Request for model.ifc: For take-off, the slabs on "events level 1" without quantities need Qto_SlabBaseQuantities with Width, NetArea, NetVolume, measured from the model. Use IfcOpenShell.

First a look at what the model holds.

```python
import ifcopenshell
import ifcopenshell.util.element
import ifcopenshell.util.unit

model = ifcopenshell.open("model.ifc")
print(model.schema)
for unit_type in ("LENGTHUNIT", "AREAUNIT", "VOLUMEUNIT"):
    print(unit_type, ifcopenshell.util.unit.calculate_unit_scale(model, unit_type))
storey = next(s for s in model.by_type("IfcBuildingStorey") if s.Name == "events level 1")
slabs = [e for e in ifcopenshell.util.element.get_decomposition(storey) if e.is_a("IfcSlab")]
for e in sorted(slabs, key=lambda e: e.id()):
    print(e.id(), e.is_a(), e.Name, list(ifcopenshell.util.element.get_psets(e, qtos_only=True)), sep=" | ")
```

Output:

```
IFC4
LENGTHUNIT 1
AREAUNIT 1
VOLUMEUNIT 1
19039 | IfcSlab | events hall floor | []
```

```python
import ifcopenshell
import ifcopenshell.api.pset
import ifcopenshell.geom
import ifcopenshell.util.element
import ifcopenshell.util.shape
import ifcopenshell.util.unit

model = ifcopenshell.open("model.ifc")
unit_scale = ifcopenshell.util.unit.calculate_unit_scale(model)
area_scale = ifcopenshell.util.unit.calculate_unit_scale(model, "AREAUNIT")
volume_scale = ifcopenshell.util.unit.calculate_unit_scale(model, "VOLUMEUNIT")
settings = ifcopenshell.geom.settings()

storey = next(s for s in model.by_type("IfcBuildingStorey") if s.Name == "events level 1")
slabs = [e for e in ifcopenshell.util.element.get_decomposition(storey) if e.is_a("IfcSlab")]

for e in sorted(slabs, key=lambda e: e.id()):
    if ifcopenshell.util.element.get_psets(e, qtos_only=True, should_inherit=False):
        continue
    # Geometry comes back in metres, in the element's own axes.
    shape = ifcopenshell.geom.create_shape(settings, e)
    values = {
        "Width": ifcopenshell.util.shape.get_z(shape.geometry) / unit_scale,
        "NetArea": ifcopenshell.util.shape.get_footprint_area(shape.geometry) / area_scale,
        "NetVolume": ifcopenshell.util.shape.get_volume(shape.geometry) / volume_scale,
    }
    qto = ifcopenshell.api.pset.add_qto(model, product=e, name="Qto_SlabBaseQuantities")
    ifcopenshell.api.pset.edit_qto(model, qto=qto, properties=values)
    print(e.id(), {k: round(v, 3) for k, v in values.items()})

model.write("model_rev.ifc")
```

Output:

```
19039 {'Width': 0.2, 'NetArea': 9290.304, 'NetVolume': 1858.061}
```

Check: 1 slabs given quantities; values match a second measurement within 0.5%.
